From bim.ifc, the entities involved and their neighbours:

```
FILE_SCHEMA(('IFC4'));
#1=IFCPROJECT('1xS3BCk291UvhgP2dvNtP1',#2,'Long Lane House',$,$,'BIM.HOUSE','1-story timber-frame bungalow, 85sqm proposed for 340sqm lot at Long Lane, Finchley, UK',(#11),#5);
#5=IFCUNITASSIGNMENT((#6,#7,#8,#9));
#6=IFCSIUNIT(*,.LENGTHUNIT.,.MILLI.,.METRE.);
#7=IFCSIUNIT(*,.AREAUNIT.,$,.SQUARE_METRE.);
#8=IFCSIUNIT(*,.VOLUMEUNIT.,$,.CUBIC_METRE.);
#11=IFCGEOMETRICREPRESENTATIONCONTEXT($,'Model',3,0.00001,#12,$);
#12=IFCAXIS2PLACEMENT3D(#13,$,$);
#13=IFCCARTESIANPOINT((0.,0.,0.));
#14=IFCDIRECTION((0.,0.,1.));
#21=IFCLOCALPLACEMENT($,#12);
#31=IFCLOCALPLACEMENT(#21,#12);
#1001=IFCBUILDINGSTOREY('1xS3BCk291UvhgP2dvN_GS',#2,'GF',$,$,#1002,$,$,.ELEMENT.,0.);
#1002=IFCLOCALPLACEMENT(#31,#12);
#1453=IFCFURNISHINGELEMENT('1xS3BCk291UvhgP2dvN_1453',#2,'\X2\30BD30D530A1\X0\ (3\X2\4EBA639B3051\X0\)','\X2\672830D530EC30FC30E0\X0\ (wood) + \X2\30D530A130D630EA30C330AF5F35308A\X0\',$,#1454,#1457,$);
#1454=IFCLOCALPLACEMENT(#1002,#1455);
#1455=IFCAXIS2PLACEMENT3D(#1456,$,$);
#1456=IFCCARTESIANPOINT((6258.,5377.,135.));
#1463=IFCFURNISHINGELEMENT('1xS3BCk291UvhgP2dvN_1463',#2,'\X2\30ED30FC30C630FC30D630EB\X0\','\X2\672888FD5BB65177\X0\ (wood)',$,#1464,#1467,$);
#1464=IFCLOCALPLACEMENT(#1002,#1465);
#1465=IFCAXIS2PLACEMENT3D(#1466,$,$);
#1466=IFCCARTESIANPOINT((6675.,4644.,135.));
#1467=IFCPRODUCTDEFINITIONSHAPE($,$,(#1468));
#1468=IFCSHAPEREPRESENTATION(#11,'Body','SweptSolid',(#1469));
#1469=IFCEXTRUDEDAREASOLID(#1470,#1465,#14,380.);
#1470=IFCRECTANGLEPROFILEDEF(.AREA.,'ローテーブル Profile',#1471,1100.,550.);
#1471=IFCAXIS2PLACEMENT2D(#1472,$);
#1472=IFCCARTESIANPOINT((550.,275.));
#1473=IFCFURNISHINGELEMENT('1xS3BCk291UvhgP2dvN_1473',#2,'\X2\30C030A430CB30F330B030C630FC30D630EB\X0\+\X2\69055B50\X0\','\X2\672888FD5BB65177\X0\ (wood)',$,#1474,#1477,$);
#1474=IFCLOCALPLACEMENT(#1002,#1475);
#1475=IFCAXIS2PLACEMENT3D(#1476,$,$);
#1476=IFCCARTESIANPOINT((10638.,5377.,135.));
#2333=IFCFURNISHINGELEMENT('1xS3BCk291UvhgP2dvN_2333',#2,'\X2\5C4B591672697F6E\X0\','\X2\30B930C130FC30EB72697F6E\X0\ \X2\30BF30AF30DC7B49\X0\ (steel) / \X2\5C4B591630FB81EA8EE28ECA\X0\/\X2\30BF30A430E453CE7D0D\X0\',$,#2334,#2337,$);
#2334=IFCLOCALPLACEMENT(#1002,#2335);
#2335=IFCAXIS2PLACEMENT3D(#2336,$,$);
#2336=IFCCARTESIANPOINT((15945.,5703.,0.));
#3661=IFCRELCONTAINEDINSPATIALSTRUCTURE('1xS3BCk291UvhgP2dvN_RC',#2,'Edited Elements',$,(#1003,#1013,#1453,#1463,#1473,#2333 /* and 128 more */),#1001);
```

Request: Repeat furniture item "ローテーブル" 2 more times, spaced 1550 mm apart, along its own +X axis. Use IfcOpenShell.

```python
import ifcopenshell
import ifcopenshell.api.geometry
import ifcopenshell.api.root
import ifcopenshell.util.element
import ifcopenshell.util.placement
import ifcopenshell.util.unit

model = ifcopenshell.open("bim.ifc")
unit_scale = ifcopenshell.util.unit.calculate_unit_scale(model)


def reuse_history(source, copy):
    """copy_class also copies each property set's owner history, people and application; keep the originals."""
    for rel in copy.IsDefinedBy:
        if rel.is_a("IfcRelDefinesByProperties") and (history := rel.RelatingPropertyDefinition.OwnerHistory):
            rel.RelatingPropertyDefinition.OwnerHistory = source.OwnerHistory
            ifcopenshell.util.element.remove_deep2(model, history)


source = model.by_guid("1xS3BCk291UvhgP2dvN_1463")
base = ifcopenshell.util.placement.get_local_placement(source.ObjectPlacement)
step = base[:3, 0] * 1.55 / unit_scale

for i in range(1, 3):
    copy = ifcopenshell.api.root.copy_class(model, product=source)
    copy.Representation = ifcopenshell.util.element.copy_deep(
        model, source.Representation, exclude=["IfcGeometricRepresentationContext", "IfcRepresentationMap"]
    )
    reuse_history(source, copy)
    matrix = base.copy()
    matrix[:3, 3] += i * step
    print("added at", matrix[:3, 3].round(3) + 0.0)
    ifcopenshell.api.geometry.edit_object_placement(model, product=copy, matrix=matrix, is_si=False)

model.write("bim_edited.ifc")
```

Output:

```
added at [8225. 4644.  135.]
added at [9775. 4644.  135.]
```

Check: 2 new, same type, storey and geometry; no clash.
